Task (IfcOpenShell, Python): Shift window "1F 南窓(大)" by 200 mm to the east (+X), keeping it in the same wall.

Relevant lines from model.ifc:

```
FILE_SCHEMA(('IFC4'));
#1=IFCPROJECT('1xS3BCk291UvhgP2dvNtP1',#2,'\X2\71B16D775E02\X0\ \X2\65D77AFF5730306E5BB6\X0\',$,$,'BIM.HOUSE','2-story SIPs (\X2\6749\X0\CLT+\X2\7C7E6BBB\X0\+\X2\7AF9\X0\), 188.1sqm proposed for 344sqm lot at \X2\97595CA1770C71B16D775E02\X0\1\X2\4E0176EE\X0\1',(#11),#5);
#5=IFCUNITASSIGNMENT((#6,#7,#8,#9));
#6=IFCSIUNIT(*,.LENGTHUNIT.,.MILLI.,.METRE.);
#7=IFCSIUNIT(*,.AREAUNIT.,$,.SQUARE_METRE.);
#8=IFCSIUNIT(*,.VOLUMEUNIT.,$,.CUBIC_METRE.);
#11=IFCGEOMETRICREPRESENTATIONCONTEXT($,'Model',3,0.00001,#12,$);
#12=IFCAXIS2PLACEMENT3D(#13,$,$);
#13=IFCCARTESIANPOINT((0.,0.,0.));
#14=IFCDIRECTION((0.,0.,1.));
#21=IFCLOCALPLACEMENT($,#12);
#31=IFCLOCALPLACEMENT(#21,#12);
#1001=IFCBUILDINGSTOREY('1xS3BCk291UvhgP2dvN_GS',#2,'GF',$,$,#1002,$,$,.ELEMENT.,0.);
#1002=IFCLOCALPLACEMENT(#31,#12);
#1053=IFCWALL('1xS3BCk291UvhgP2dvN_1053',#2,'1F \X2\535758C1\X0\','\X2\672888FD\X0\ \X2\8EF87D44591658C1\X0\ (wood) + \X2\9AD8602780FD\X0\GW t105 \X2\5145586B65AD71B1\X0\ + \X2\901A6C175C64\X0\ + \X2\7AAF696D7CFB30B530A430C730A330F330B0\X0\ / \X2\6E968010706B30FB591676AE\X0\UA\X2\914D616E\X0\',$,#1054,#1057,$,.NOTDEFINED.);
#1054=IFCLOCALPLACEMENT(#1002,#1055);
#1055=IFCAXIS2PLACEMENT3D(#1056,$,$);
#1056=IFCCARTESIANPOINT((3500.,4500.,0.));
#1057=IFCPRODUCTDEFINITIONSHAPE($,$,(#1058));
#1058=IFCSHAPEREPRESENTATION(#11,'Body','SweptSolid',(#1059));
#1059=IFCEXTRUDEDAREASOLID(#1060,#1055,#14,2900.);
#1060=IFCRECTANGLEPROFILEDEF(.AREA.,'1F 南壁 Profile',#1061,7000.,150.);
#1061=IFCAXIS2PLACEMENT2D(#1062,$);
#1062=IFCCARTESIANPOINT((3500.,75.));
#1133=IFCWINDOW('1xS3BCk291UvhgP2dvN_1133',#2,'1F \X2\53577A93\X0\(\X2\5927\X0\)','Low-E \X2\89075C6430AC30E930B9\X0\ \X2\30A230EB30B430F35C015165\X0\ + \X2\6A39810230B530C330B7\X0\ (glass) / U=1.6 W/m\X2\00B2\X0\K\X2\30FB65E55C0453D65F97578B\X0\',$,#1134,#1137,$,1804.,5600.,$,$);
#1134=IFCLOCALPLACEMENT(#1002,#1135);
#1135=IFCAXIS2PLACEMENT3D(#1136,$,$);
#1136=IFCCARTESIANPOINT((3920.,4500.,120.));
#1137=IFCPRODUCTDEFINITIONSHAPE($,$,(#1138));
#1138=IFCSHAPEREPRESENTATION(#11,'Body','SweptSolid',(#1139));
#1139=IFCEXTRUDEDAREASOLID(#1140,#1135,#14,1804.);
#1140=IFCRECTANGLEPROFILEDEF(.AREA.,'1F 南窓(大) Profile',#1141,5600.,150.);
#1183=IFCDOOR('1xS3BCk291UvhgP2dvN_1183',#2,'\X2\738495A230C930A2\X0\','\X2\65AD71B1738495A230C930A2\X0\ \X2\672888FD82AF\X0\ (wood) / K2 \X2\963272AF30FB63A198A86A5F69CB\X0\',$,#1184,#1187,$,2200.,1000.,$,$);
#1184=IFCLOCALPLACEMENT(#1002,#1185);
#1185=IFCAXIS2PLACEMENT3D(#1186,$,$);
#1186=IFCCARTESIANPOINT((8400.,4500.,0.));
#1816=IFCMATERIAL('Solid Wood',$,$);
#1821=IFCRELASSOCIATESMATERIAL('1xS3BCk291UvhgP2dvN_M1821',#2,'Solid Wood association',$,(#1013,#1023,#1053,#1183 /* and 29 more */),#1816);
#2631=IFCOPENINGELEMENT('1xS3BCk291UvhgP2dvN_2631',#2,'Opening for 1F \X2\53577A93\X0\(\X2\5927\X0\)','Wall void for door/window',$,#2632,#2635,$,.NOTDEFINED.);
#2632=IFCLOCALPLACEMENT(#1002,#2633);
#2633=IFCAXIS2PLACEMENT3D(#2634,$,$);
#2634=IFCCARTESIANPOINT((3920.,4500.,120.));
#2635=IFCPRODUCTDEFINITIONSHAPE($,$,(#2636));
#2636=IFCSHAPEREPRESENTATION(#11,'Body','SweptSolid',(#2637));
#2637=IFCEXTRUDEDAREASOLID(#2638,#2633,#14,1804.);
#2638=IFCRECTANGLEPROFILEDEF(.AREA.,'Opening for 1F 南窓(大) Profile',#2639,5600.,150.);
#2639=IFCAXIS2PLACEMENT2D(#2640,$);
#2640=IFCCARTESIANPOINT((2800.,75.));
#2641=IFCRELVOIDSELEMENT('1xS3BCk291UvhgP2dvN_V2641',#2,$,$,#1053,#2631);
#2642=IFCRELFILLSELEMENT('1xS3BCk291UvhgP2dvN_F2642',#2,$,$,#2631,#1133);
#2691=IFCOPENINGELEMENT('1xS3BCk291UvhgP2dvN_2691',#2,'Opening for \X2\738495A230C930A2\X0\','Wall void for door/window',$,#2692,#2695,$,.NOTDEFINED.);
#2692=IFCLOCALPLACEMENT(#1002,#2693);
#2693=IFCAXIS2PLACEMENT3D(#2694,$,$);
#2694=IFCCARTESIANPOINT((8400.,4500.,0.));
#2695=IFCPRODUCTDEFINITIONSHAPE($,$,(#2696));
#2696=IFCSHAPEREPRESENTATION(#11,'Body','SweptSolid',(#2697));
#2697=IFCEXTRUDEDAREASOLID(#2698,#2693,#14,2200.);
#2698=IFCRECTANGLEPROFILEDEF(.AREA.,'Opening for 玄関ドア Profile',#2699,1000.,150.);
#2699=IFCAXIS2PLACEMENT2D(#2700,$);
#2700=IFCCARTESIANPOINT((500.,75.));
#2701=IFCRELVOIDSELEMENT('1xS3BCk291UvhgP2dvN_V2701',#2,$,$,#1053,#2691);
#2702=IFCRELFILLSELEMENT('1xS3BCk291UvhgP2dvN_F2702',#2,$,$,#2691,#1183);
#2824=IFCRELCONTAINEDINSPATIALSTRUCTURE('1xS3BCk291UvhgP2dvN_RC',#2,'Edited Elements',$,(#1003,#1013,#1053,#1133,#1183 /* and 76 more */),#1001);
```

```python
import ifcopenshell
import ifcopenshell.api.geometry
import ifcopenshell.util.placement

model = ifcopenshell.open("model.ifc")

window = model.by_guid("1xS3BCk291UvhgP2dvN_1133")
opening = window.FillsVoids[0].RelatingOpeningElement
wall = opening.VoidsElements[0].RelatingBuildingElement

wall_matrix = ifcopenshell.util.placement.get_local_placement(wall.ObjectPlacement)
shift = wall_matrix[:3, 0] * 200.0
before = ifcopenshell.util.placement.get_local_placement(window.ObjectPlacement)[:3, 3].copy()

# The window is not placed relative to its opening, so move both.
for product in (opening, window):
    matrix = ifcopenshell.util.placement.get_local_placement(product.ObjectPlacement)
    matrix[:3, 3] += shift
    ifcopenshell.api.geometry.edit_object_placement(model, product=product, matrix=matrix, is_si=False)

after = ifcopenshell.util.placement.get_local_placement(window.ObjectPlacement)[:3, 3]
print("window moved by", (after - before).round(3) + 0.0)

model.write("model_edited.ifc")
```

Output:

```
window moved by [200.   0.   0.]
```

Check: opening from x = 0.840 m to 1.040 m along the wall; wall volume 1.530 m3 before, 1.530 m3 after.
